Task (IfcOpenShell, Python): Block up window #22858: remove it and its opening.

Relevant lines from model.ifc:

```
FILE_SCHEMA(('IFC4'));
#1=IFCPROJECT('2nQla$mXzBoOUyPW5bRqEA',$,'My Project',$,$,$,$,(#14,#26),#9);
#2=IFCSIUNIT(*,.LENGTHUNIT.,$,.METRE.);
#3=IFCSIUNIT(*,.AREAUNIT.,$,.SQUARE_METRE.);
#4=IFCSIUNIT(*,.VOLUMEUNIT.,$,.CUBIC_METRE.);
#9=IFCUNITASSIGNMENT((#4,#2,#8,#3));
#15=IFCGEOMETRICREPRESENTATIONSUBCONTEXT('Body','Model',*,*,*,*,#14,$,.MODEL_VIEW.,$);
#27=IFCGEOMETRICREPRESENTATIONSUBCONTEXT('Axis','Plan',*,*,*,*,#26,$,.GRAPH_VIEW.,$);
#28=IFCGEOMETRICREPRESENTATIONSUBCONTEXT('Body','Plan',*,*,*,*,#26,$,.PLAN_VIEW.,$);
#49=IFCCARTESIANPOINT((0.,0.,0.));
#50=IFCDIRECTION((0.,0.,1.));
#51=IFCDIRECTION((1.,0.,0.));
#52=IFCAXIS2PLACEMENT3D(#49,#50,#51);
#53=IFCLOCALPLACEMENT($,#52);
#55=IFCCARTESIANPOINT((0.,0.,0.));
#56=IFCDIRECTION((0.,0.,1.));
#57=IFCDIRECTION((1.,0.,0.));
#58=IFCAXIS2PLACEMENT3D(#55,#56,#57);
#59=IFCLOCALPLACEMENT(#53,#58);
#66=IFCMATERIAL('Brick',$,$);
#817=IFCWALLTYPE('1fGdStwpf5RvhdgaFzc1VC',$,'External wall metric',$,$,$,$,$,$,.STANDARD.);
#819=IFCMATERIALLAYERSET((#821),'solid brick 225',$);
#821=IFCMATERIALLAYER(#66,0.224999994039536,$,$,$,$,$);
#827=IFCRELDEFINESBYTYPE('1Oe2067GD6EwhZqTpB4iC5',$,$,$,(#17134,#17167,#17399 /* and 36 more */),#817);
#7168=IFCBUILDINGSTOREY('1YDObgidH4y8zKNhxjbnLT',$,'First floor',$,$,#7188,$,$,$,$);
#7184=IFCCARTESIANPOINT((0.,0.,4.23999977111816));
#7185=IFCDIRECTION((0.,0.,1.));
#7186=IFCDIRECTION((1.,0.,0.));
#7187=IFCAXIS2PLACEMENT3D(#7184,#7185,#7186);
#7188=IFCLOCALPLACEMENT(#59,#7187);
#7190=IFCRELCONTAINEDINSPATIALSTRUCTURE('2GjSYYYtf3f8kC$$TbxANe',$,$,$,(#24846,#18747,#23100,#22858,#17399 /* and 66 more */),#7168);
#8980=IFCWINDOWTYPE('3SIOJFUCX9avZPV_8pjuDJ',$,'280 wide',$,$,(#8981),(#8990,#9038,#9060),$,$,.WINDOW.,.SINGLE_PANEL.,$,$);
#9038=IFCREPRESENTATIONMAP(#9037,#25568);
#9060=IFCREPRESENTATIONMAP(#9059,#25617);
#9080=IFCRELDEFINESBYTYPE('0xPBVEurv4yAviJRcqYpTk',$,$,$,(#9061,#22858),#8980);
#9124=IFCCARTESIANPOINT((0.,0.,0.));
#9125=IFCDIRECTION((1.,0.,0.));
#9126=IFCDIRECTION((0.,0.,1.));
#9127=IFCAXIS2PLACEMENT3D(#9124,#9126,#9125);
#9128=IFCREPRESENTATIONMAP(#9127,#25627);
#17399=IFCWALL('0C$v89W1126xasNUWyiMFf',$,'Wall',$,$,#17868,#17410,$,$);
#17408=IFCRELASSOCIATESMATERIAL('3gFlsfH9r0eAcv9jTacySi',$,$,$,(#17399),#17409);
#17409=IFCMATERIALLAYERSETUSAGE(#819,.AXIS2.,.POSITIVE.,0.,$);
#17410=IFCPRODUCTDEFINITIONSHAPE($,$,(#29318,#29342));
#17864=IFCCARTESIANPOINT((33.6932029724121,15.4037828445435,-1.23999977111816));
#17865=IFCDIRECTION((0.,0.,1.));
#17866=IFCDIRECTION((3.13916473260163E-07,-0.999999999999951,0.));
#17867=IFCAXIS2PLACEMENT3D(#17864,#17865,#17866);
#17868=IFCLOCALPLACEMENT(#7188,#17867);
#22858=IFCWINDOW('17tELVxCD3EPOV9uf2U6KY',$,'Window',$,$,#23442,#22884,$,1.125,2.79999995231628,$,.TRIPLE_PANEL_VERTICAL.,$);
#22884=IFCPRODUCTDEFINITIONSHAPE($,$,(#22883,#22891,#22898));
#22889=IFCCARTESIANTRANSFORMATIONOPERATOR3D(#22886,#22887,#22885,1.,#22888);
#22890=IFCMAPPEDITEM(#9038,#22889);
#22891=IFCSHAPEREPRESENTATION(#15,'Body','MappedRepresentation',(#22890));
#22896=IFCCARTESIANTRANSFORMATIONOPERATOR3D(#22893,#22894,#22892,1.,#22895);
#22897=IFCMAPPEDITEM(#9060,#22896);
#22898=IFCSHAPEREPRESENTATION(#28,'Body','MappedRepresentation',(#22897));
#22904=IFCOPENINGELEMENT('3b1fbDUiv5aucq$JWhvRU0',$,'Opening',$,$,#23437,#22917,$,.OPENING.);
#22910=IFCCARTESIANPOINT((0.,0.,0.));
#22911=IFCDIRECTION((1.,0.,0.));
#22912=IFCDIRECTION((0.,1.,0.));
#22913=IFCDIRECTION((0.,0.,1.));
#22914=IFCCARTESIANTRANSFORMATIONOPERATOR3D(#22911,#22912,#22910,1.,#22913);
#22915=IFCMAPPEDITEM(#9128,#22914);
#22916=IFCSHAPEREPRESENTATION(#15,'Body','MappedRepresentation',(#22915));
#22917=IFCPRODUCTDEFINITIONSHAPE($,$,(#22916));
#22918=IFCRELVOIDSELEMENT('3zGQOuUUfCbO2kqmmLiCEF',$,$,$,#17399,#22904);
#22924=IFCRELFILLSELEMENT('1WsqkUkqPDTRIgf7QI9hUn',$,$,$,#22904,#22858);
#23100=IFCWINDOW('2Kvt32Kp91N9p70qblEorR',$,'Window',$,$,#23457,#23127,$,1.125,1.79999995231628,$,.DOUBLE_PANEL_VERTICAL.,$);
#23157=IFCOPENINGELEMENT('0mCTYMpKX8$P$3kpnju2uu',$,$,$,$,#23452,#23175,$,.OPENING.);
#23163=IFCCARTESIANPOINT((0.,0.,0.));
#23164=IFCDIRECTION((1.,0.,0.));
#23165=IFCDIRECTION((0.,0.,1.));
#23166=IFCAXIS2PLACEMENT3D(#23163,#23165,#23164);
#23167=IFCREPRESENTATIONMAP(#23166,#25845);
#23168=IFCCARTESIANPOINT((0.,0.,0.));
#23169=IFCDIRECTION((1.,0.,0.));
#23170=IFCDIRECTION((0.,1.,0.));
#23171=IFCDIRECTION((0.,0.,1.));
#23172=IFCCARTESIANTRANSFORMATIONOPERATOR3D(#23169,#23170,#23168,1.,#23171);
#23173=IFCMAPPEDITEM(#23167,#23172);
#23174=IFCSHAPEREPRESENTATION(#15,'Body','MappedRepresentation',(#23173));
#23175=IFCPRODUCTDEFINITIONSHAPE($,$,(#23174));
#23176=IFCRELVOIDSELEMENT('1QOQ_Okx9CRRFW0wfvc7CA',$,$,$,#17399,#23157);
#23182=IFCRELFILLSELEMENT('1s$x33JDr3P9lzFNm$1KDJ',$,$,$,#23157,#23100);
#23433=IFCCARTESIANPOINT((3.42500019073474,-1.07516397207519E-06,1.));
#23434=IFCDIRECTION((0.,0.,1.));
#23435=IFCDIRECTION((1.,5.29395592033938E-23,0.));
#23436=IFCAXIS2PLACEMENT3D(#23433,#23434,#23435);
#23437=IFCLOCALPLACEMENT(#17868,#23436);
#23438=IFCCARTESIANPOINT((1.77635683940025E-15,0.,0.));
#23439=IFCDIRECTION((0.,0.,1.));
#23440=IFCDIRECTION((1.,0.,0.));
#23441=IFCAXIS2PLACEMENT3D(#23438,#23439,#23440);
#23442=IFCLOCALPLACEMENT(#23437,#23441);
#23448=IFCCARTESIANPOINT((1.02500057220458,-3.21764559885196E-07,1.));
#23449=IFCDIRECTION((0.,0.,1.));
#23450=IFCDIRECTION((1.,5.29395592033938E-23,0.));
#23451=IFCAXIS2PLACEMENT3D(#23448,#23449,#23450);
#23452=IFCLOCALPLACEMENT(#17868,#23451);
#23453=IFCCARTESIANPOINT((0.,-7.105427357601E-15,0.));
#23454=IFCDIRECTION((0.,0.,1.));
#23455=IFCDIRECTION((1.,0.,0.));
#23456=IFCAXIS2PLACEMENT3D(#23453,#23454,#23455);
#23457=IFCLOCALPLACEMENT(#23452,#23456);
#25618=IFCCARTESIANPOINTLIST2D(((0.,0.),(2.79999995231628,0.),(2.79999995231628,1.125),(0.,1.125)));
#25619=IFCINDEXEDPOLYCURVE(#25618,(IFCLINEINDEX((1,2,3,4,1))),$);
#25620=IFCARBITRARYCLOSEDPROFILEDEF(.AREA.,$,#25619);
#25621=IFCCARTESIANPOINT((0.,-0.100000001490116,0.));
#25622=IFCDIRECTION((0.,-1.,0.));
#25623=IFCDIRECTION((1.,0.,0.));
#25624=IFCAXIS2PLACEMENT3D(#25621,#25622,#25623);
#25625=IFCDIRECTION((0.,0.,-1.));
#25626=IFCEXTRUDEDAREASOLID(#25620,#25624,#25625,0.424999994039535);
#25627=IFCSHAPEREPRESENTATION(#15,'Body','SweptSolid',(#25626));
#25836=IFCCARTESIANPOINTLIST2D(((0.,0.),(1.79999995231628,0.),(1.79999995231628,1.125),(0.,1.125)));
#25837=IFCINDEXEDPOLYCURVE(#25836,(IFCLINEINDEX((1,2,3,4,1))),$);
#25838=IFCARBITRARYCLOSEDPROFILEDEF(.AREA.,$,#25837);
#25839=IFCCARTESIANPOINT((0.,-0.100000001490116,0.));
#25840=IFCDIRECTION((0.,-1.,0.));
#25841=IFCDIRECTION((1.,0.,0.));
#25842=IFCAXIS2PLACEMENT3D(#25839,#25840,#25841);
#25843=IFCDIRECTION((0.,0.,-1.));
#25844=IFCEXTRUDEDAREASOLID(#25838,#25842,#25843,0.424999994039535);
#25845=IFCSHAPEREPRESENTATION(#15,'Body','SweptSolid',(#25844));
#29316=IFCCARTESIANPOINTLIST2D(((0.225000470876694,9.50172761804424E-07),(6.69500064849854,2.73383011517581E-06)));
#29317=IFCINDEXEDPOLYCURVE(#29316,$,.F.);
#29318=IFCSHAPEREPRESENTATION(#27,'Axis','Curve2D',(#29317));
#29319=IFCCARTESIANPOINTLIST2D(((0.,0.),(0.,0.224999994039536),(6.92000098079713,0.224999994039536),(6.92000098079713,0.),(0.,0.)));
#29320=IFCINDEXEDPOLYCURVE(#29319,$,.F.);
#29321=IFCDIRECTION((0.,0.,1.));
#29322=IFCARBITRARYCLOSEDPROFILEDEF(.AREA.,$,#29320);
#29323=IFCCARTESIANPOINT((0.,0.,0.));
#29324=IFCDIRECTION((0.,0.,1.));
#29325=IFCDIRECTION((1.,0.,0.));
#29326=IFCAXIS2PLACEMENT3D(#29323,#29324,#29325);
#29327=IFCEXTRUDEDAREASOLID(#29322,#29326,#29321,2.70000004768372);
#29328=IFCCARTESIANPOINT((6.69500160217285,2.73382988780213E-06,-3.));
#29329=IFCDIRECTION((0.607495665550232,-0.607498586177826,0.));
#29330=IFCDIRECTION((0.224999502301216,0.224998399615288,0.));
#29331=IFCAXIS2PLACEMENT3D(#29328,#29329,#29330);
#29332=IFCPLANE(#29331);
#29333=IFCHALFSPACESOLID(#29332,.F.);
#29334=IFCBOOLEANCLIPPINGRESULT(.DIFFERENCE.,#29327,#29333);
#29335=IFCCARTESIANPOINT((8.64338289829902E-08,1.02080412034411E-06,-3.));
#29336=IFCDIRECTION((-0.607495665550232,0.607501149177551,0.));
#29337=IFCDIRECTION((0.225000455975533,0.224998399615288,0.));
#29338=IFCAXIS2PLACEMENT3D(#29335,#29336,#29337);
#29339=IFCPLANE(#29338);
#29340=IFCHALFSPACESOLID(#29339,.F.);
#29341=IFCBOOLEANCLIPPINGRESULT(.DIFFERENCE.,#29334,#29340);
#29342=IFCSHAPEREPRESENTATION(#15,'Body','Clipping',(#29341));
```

```python
import ifcopenshell
import ifcopenshell.api.feature
import ifcopenshell.api.root
import ifcopenshell.geom
import ifcopenshell.util.shape

model = ifcopenshell.open("model.ifc")
settings = ifcopenshell.geom.settings()


def volume(element):
    """Net volume in cubic metres, openings subtracted."""
    shape = ifcopenshell.geom.create_shape(settings, element)
    return ifcopenshell.util.shape.get_volume(shape.geometry)


window = model.by_guid("17tELVxCD3EPOV9uf2U6KY")
opening = window.FillsVoids[0].RelatingOpeningElement
wall = opening.VoidsElements[0].RelatingBuildingElement
before = volume(wall)

ifcopenshell.api.root.remove_product(model, product=window)
ifcopenshell.api.feature.remove_feature(model, feature=opening)

after = volume(wall)

print(f"wall volume {before:.3f} -> {after:.3f} m3")

model.write("model-out.ifc")
```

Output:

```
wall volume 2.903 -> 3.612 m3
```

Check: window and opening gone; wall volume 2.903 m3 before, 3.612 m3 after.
